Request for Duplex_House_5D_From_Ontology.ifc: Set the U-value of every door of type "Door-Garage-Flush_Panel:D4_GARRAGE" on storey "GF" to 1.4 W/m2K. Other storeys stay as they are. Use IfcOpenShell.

First a look at what the model holds.

```python
import ifcopenshell
import ifcopenshell.util.element

model = ifcopenshell.open("Duplex_House_5D_From_Ontology.ifc")
print(model.schema)
storey = next(s for s in model.by_type("IfcBuildingStorey") if s.Name == "GF")
doors = [e for e in ifcopenshell.util.element.get_decomposition(storey) if e.is_a("IfcDoor")]
seen = {}
for e in doors:
    element_type = ifcopenshell.util.element.get_type(e)
    key = (element_type.Name if element_type != e and element_type else None, ifcopenshell.util.element.get_pset(e, "Pset_DoorCommon", "ThermalTransmittance"))
    seen[key] = seen.get(key, 0) + 1
for (name, value), count in sorted(seen.items(), key=str):
    print(count, "x", name, "|", value)
```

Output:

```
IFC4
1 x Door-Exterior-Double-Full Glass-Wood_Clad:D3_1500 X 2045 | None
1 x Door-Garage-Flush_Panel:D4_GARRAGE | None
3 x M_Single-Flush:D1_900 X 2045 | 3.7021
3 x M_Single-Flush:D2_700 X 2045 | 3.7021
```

```python
import ifcopenshell
import ifcopenshell.api.pset
import ifcopenshell.util.element

model = ifcopenshell.open("Duplex_House_5D_From_Ontology.ifc")

storey = next(s for s in model.by_type("IfcBuildingStorey") if s.Name == "GF")
doors = [e for e in ifcopenshell.util.element.get_decomposition(storey) if e.is_a("IfcDoor")]

count = 0
for e in doors:
    element_type = ifcopenshell.util.element.get_type(e)
    if element_type in (None, e) or element_type.Name != "Door-Garage-Flush_Panel:D4_GARRAGE":
        continue
    # add_pset returns the element's existing set when there is one.
    pset = ifcopenshell.api.pset.add_pset(model, product=e, name="Pset_DoorCommon")
    ifcopenshell.api.pset.edit_pset(model, pset=pset, properties={"ThermalTransmittance": 1.4})
    count += 1

print(count, "doors updated")

model.write("Duplex_House_5D_From_Ontology_edited.ifc")
```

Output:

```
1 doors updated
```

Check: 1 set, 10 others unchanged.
